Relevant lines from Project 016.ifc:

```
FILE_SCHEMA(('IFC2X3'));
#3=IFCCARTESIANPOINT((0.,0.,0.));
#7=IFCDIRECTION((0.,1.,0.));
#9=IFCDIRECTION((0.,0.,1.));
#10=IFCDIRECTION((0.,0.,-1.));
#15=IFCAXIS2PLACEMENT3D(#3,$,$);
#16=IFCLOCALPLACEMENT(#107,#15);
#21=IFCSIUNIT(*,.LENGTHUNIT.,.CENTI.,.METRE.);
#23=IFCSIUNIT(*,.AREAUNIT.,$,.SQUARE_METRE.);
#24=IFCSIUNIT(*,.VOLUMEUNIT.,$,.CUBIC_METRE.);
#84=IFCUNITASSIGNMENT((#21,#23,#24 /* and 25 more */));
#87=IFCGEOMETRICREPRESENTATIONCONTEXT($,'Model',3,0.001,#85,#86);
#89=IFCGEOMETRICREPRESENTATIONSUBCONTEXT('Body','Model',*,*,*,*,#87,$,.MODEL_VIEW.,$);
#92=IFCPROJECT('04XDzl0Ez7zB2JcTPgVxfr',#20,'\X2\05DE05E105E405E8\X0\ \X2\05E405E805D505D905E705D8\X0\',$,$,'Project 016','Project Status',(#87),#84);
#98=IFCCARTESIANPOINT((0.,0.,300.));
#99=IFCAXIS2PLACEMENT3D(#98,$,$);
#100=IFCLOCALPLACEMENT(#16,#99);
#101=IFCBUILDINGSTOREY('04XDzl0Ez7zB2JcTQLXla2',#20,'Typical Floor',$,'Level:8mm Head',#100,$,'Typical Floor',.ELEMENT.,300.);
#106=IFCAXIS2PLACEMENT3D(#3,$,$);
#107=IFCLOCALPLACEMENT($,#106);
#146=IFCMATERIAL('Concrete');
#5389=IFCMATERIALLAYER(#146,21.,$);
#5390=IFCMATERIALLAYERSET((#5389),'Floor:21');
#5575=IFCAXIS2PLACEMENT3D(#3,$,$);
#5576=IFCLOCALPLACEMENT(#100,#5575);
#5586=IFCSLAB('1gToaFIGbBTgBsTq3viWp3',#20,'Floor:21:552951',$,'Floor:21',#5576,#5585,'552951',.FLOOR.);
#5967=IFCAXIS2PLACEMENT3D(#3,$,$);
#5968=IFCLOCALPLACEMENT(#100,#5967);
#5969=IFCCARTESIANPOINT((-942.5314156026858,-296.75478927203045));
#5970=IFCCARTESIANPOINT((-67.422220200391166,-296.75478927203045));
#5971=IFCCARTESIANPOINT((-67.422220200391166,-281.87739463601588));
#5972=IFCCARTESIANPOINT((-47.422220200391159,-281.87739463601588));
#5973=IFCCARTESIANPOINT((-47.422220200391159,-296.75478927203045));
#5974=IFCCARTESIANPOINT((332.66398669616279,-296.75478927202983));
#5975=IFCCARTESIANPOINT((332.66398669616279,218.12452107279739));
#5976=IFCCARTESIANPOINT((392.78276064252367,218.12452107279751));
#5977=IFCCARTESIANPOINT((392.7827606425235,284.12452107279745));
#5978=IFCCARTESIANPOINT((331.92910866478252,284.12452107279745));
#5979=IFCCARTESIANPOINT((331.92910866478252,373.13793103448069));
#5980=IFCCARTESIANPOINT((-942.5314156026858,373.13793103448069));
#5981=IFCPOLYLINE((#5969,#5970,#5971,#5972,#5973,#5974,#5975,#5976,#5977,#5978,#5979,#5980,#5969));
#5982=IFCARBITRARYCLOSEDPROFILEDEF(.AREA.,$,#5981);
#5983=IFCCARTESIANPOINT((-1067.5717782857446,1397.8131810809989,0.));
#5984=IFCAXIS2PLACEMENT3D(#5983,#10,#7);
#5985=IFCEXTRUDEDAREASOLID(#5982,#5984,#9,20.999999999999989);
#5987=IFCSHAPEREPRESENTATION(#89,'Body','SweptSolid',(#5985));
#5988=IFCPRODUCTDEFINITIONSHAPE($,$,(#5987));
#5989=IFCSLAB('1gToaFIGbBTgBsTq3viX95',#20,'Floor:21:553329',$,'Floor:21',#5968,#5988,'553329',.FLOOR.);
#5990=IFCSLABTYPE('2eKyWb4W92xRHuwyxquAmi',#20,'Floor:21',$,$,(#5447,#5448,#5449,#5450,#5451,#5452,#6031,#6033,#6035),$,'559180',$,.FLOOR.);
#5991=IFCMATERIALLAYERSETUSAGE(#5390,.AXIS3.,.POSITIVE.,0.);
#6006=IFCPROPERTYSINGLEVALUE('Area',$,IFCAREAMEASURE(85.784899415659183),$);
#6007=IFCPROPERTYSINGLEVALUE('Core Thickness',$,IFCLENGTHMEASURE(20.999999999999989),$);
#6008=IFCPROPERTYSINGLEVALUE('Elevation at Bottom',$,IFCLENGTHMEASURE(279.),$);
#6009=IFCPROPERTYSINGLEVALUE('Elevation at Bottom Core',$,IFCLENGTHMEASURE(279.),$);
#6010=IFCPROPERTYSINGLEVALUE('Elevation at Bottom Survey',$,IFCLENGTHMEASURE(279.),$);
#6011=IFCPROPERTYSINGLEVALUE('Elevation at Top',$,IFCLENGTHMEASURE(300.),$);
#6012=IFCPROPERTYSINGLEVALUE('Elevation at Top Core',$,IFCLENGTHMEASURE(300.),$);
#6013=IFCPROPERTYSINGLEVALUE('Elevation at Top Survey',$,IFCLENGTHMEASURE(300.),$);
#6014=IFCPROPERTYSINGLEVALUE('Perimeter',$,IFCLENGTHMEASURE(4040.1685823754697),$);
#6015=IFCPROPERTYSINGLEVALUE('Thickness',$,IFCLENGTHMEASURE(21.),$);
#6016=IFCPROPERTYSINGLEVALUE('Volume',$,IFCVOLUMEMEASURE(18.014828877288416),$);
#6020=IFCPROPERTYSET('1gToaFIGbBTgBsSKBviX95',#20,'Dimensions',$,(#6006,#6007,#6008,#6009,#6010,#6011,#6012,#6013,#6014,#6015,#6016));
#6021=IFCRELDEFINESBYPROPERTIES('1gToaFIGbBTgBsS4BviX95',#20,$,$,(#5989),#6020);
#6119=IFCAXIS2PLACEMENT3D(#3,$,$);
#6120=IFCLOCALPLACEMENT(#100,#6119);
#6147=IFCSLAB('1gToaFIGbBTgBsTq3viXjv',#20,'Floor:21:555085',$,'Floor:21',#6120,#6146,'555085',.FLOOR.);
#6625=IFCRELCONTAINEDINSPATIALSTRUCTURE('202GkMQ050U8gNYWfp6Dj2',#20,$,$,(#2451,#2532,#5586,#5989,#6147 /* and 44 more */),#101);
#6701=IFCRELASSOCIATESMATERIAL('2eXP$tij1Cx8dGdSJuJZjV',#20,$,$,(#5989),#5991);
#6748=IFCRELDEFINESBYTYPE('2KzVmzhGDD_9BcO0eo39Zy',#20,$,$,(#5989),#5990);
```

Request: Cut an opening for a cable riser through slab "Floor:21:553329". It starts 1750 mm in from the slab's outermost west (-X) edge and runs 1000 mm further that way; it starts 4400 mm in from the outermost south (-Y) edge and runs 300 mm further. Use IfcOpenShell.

```python
import numpy as np
import ifcopenshell
import ifcopenshell.api.feature
import ifcopenshell.api.geometry
import ifcopenshell.api.pset
import ifcopenshell.api.root
import ifcopenshell.geom
import ifcopenshell.util.element
import ifcopenshell.util.placement
import ifcopenshell.util.representation
import ifcopenshell.util.shape
import ifcopenshell.util.unit

model = ifcopenshell.open("Project 016.ifc")
unit_scale = ifcopenshell.util.unit.calculate_unit_scale(model)
area_scale = ifcopenshell.util.unit.calculate_unit_scale(model, "AREAUNIT")
volume_scale = ifcopenshell.util.unit.calculate_unit_scale(model, "VOLUMEUNIT")
settings = ifcopenshell.geom.settings()


def volume(element):
    """Net volume in cubic metres, openings subtracted."""
    shape = ifcopenshell.geom.create_shape(settings, element)
    return ifcopenshell.util.shape.get_volume(shape.geometry)


slab = model.by_guid("1gToaFIGbBTgBsTq3viX95")
before = volume(slab)

# Extent in the slab's own axes, in metres. The edges named are its -X and -Y sides.
slab_shape = ifcopenshell.geom.create_shape(settings, slab)
vertices = ifcopenshell.util.shape.get_vertices(slab_shape.geometry)
x_min, y_min, bottom = vertices.min(axis=0)
top = vertices[:, 2].max()

opening = ifcopenshell.api.root.create_entity(model, ifc_class="IfcOpeningElement", name="Cable riser opening")
context = ifcopenshell.util.representation.get_context(model, "Model", "Body", "MODEL_VIEW")
width, depth = 1, 0.3
outline = [(0.0, 0.0), (width, 0.0), (width, depth), (0.0, depth), (0.0, 0.0)]
# Overshoot both faces by 50 mm so the cut is clean.
shape = ifcopenshell.api.geometry.add_slab_representation(
    model, context=context, depth=top - bottom + 0.1, polyline=outline
)
ifcopenshell.api.geometry.assign_representation(model, product=opening, representation=shape)

matrix = ifcopenshell.util.placement.get_local_placement(slab.ObjectPlacement)
matrix[:, 3] = matrix @ np.append(np.array([x_min + 1.75, y_min + 4.4, bottom - 0.05]) / unit_scale, 1.0)
ifcopenshell.api.geometry.edit_object_placement(model, product=opening, matrix=matrix, is_si=False)
ifcopenshell.api.feature.add_feature(model, feature=opening, element=slab)

after = volume(slab)

# Update the slab's stored quantities.
pset = model.by_id(ifcopenshell.util.element.get_pset(slab, "Dimensions", should_inherit=False)["id"])
ifcopenshell.api.pset.edit_pset(model, pset=pset, properties={
    "Area": model.create_entity("IfcAreaMeasure", after / (top - bottom) / area_scale),
    "Volume": model.create_entity("IfcVolumeMeasure", after / volume_scale),
})

print(f"slab volume {before:.3f} -> {after:.3f} m3")

model.write("Project 016_rev.ifc")
```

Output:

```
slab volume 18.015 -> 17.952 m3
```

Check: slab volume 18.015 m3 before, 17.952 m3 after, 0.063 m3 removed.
